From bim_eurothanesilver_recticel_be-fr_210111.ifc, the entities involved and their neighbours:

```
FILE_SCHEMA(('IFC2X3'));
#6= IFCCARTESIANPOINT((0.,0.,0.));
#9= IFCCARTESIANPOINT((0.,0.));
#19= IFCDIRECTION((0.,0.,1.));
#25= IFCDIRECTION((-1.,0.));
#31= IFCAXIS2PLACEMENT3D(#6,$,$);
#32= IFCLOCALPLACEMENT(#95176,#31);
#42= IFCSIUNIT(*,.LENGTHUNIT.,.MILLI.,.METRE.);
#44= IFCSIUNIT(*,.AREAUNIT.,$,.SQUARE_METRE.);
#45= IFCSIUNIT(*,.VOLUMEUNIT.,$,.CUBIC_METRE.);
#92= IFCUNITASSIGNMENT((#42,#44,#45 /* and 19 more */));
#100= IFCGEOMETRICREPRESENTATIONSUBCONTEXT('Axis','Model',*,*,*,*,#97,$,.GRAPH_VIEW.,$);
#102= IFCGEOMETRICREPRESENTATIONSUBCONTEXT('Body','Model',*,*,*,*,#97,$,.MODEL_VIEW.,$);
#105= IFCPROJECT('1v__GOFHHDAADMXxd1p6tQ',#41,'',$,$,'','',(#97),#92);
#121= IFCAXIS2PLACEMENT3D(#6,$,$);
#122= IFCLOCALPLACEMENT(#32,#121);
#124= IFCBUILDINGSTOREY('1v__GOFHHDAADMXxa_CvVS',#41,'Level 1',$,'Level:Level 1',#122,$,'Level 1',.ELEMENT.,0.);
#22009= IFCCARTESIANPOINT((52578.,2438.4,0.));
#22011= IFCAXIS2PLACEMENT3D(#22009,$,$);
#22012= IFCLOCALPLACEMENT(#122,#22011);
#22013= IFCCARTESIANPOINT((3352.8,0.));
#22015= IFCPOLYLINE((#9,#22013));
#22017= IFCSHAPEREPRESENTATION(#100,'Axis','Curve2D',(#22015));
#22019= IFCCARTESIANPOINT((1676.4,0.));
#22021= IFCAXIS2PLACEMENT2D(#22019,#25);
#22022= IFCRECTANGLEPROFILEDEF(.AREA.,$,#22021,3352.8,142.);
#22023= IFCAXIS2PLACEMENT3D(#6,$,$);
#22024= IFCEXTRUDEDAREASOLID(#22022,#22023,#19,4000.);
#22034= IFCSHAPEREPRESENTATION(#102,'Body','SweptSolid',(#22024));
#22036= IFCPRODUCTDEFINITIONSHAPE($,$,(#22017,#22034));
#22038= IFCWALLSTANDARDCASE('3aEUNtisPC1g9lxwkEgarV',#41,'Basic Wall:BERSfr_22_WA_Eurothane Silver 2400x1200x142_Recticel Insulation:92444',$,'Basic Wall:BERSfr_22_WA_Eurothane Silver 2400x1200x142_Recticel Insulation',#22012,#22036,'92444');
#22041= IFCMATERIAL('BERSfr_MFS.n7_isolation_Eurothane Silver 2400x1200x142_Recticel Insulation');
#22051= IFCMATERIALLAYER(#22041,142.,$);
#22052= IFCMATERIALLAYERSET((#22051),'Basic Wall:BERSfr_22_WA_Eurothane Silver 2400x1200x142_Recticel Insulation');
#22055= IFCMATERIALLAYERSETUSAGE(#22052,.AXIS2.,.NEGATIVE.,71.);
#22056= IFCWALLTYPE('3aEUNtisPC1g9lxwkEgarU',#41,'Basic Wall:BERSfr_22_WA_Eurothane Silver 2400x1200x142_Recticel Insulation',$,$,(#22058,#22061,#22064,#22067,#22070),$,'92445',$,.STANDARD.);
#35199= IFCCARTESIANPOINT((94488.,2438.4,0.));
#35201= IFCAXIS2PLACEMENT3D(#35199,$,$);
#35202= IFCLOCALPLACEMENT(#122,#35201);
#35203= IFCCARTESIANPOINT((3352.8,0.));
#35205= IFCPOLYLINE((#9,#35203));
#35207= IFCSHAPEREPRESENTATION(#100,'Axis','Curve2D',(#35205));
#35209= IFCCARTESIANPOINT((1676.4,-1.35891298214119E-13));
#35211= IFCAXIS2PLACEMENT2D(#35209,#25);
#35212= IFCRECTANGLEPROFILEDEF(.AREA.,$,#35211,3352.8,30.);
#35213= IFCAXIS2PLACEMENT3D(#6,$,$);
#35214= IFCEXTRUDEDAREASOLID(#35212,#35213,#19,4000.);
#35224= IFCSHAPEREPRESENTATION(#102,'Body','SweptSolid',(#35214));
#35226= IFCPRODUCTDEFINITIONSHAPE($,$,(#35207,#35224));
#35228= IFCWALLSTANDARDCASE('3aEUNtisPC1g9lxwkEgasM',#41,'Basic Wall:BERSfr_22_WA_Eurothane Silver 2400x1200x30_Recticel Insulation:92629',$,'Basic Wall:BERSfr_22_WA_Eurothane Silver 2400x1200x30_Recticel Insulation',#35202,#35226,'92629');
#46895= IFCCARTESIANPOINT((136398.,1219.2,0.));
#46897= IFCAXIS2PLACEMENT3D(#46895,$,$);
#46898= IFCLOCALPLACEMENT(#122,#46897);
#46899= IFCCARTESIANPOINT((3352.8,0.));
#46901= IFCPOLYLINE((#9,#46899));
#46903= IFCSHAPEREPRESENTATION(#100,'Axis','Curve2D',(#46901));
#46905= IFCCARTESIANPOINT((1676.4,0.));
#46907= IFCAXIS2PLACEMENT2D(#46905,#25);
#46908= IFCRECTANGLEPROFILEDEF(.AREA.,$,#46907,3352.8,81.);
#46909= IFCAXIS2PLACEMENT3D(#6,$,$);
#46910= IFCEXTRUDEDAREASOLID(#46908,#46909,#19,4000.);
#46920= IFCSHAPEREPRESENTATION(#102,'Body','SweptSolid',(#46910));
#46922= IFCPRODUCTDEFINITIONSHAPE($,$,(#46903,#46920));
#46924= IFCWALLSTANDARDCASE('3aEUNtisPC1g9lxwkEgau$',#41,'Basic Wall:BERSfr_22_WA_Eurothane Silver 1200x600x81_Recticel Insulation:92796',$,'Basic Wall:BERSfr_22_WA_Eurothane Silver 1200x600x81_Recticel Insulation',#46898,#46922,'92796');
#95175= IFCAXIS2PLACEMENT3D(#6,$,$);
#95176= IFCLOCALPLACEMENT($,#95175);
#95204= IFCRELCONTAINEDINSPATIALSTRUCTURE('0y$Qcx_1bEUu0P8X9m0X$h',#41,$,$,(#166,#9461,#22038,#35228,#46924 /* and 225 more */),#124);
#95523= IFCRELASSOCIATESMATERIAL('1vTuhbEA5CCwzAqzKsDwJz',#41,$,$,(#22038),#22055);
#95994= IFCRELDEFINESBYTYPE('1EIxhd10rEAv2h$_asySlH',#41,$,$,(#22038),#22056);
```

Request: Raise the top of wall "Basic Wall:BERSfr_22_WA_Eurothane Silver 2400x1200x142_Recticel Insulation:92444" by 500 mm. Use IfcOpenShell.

```python
import ifcopenshell
import ifcopenshell.geom
import ifcopenshell.util.representation
import ifcopenshell.util.shape

model = ifcopenshell.open("bim_eurothanesilver_recticel_be-fr_210111.ifc")
settings = ifcopenshell.geom.settings()


def volume(element):
    """Net volume in cubic metres, openings subtracted."""
    shape = ifcopenshell.geom.create_shape(settings, element)
    return ifcopenshell.util.shape.get_volume(shape.geometry)


wall = model.by_guid("3aEUNtisPC1g9lxwkEgarV")
before = volume(wall)

body = ifcopenshell.util.representation.get_representation(wall, "Model", "Body")
solid = body.Items[0]
old_height = solid.Depth
solid.Depth += 500.0
after = volume(wall)

print(f"height {old_height:g} -> {solid.Depth:g}, volume {before:.3f} -> {after:.3f} m3")

model.write("bim_eurothanesilver_recticel_be-fr_210111_updated.ifc")
```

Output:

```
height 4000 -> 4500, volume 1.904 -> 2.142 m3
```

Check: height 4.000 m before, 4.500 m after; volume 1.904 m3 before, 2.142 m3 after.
